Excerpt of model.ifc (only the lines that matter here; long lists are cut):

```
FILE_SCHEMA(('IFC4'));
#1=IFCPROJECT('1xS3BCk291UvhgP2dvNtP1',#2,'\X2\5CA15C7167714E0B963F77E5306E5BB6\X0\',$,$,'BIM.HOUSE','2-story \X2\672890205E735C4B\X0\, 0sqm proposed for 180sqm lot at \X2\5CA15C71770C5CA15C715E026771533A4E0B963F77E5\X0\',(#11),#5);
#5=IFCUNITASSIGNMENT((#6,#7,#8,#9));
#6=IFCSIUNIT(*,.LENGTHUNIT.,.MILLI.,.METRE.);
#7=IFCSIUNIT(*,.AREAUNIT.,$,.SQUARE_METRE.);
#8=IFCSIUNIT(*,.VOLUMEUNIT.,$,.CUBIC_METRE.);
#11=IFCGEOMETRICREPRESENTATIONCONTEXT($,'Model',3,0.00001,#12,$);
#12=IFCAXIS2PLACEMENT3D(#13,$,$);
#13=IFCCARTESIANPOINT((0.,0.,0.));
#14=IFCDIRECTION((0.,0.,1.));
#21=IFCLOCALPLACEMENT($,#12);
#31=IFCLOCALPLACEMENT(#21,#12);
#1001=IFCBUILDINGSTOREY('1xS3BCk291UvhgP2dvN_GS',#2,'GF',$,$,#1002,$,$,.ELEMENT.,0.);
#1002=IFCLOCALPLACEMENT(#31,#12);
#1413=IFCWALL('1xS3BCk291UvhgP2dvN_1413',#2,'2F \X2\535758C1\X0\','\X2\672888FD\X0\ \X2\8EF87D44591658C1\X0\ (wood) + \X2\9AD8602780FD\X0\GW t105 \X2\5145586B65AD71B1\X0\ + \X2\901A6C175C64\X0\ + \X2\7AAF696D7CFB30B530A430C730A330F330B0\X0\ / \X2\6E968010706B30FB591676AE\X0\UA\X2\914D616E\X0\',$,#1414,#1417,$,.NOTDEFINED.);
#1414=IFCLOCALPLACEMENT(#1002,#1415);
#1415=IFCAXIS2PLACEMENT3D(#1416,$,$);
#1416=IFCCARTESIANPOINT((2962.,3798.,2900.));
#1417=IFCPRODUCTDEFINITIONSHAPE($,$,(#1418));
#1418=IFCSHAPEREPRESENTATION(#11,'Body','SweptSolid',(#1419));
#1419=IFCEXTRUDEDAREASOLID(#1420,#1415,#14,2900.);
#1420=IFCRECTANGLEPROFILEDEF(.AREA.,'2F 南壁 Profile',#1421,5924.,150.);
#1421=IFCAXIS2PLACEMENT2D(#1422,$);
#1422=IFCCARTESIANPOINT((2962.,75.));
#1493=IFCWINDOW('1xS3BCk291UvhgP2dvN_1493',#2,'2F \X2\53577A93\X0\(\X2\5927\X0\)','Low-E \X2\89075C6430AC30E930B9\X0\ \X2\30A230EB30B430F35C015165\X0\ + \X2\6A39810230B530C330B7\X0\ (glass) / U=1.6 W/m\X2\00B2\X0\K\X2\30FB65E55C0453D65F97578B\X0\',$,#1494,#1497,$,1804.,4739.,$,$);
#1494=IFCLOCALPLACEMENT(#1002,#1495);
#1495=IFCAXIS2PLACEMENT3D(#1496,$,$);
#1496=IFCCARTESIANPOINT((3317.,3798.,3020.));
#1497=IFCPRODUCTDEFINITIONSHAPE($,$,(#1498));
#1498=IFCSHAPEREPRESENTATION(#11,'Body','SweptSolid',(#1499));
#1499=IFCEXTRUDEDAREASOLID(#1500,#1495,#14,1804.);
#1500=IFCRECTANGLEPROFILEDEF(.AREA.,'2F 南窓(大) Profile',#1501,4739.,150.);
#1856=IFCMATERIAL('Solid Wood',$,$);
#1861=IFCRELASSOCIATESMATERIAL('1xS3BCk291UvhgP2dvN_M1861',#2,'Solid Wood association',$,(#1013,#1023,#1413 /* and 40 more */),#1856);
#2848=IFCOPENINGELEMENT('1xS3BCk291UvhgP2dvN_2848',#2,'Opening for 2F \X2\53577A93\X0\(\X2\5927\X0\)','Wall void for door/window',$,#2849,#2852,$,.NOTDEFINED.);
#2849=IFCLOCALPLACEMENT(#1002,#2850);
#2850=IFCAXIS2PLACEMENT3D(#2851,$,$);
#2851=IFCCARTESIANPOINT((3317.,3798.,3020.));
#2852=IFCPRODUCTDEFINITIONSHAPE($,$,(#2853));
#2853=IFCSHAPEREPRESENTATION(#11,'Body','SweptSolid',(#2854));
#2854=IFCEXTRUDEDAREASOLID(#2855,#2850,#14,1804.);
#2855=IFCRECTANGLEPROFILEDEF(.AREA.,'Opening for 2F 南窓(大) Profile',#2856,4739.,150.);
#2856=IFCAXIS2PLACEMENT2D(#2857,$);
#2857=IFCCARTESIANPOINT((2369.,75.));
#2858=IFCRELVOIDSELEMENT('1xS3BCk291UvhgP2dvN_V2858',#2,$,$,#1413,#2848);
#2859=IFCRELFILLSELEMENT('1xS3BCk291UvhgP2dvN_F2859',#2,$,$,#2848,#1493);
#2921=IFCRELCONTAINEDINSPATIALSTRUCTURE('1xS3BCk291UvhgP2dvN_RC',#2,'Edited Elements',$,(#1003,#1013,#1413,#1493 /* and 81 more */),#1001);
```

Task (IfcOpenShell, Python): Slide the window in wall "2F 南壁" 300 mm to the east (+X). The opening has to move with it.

```python
import ifcopenshell
import ifcopenshell.api.geometry
import ifcopenshell.util.placement
import ifcopenshell.util.unit

model = ifcopenshell.open("model.ifc")
unit_scale = ifcopenshell.util.unit.calculate_unit_scale(model)

window = model.by_id(1493)
opening = window.FillsVoids[0].RelatingOpeningElement
wall = opening.VoidsElements[0].RelatingBuildingElement

wall_matrix = ifcopenshell.util.placement.get_local_placement(wall.ObjectPlacement)
shift = wall_matrix[:3, 0] * 0.3 / unit_scale
before = ifcopenshell.util.placement.get_local_placement(window.ObjectPlacement)[:3, 3].copy()

# The window is not placed relative to its opening, so move both.
for product in (opening, window):
    matrix = ifcopenshell.util.placement.get_local_placement(product.ObjectPlacement)
    matrix[:3, 3] += shift
    ifcopenshell.api.geometry.edit_object_placement(model, product=product, matrix=matrix, is_si=False)

after = ifcopenshell.util.placement.get_local_placement(window.ObjectPlacement)[:3, 3]
print("window moved by", (after - before).round(3) + 0.0)

model.write("model_updated.ifc")
```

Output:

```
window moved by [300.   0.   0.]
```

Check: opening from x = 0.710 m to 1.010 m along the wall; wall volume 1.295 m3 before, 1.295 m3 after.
